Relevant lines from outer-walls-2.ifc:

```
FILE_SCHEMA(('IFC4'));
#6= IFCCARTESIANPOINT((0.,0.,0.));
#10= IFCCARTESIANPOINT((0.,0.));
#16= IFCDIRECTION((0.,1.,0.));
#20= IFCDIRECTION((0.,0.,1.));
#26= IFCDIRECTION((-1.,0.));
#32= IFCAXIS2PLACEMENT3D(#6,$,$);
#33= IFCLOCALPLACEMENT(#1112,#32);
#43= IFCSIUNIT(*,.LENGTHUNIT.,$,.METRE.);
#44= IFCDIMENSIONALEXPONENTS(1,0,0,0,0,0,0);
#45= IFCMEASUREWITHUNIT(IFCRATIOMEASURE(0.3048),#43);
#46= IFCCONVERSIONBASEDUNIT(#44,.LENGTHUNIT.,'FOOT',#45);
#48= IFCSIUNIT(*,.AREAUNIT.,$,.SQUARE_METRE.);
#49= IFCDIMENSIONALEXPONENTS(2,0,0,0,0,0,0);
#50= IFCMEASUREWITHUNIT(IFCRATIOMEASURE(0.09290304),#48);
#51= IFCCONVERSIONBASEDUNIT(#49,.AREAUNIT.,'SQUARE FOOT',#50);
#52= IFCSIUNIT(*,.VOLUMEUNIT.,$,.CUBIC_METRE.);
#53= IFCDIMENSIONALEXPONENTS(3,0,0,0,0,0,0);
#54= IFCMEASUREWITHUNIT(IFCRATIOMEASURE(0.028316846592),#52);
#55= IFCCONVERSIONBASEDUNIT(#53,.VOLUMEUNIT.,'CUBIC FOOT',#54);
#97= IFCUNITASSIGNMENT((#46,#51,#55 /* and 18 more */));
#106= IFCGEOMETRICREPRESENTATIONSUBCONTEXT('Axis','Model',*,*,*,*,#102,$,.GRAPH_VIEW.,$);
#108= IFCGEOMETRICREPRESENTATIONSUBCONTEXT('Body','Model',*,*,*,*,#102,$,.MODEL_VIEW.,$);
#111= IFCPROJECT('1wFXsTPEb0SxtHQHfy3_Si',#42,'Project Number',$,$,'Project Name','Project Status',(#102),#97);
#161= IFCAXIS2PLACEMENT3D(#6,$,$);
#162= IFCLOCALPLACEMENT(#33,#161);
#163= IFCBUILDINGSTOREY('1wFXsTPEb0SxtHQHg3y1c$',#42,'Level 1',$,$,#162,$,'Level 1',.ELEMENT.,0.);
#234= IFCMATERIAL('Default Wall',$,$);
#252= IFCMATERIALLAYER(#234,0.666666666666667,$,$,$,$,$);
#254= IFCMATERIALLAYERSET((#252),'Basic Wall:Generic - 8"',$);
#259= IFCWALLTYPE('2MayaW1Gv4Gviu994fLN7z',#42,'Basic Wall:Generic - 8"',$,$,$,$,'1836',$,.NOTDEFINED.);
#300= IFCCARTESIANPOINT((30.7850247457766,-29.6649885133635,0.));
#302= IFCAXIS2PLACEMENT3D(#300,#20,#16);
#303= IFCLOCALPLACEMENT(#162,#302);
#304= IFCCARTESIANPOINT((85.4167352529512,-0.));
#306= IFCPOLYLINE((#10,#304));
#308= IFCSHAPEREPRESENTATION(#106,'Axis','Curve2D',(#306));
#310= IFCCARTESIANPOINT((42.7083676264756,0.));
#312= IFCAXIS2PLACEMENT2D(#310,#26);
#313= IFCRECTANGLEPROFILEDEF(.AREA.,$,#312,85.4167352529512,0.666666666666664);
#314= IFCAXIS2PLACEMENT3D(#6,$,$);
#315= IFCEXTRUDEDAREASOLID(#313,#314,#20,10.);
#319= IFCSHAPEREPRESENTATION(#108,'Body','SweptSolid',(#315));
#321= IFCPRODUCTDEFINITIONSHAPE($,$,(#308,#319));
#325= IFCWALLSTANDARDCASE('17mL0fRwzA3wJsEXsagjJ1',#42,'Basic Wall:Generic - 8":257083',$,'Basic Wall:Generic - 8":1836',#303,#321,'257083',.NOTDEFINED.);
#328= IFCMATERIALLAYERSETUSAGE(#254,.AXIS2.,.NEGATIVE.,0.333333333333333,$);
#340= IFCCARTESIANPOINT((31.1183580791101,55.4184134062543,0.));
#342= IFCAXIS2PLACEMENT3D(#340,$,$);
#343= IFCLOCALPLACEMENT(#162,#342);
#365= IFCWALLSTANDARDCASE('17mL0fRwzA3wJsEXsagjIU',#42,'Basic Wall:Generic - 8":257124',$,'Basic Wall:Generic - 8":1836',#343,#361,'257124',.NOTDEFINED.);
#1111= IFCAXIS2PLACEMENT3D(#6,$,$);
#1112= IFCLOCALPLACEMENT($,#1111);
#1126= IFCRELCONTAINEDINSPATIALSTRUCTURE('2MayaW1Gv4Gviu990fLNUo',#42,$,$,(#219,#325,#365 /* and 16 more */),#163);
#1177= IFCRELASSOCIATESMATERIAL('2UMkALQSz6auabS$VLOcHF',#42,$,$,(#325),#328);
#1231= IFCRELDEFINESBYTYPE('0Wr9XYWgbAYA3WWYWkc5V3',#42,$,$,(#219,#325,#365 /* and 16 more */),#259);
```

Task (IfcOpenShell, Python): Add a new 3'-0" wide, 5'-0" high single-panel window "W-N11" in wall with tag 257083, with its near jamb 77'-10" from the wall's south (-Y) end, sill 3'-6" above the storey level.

```python
import numpy as np
import ifcopenshell
import ifcopenshell.api.feature
import ifcopenshell.api.geometry
import ifcopenshell.api.root
import ifcopenshell.api.spatial
import ifcopenshell.geom
import ifcopenshell.util.element
import ifcopenshell.util.placement
import ifcopenshell.util.representation
import ifcopenshell.util.shape
import ifcopenshell.util.unit

model = ifcopenshell.open("outer-walls-2.ifc")
unit_scale = ifcopenshell.util.unit.calculate_unit_scale(model)
settings = ifcopenshell.geom.settings()


def volume(element):
    """Net volume in cubic metres, openings subtracted."""
    shape = ifcopenshell.geom.create_shape(settings, element)
    return ifcopenshell.util.shape.get_volume(shape.geometry)


wall = model.by_guid("17mL0fRwzA3wJsEXsagjJ1")
storey = ifcopenshell.util.element.get_container(wall, ifc_class="IfcBuildingStorey")
context = ifcopenshell.util.representation.get_context(model, "Model", "Body", "MODEL_VIEW")
before = volume(wall)

width, height, from_end, sill = 0.9144, 1.524, 23.7236, 1.0668  # metres

# The wall runs along its own X axis, and the end named is its -X end.
wall_shape = ifcopenshell.geom.create_shape(settings, wall)
x, y, z = ifcopenshell.util.shape.get_vertices(wall_shape.geometry).T
start = x.min() + from_end
face, thickness = float(y.min()), float(y.max() - y.min())
wall_matrix = ifcopenshell.util.placement.get_local_placement(wall.ObjectPlacement)
level = ifcopenshell.util.placement.get_local_placement(storey.ObjectPlacement)[2, 3]


def in_wall(x, y):
    """Placement at x, y metres in the wall's axes, at sill height."""
    matrix = wall_matrix.copy()
    matrix[:, 3] = wall_matrix @ np.array([x / unit_scale, y / unit_scale, 0.0, 1.0])
    matrix[2, 3] = level + sill / unit_scale
    return matrix


# Opening: a box that overshoots both wall faces by 50 mm.
opening = ifcopenshell.api.root.create_entity(model, ifc_class="IfcOpeningElement", predefined_type="OPENING")
box = ifcopenshell.api.geometry.add_wall_representation(
    model, context=context, length=width, height=height, thickness=thickness + 0.1
)
ifcopenshell.api.geometry.assign_representation(model, product=opening, representation=box)
ifcopenshell.api.geometry.edit_object_placement(model, product=opening, matrix=in_wall(start, face - 0.05), is_si=False)
ifcopenshell.api.feature.add_feature(model, feature=opening, element=wall)

window = ifcopenshell.api.root.create_entity(model, ifc_class="IfcWindow", name="W-N11", predefined_type="WINDOW")
window.OverallWidth, window.OverallHeight = width / unit_scale, height / unit_scale
window.PartitioningType = "SINGLE_PANEL"
body = ifcopenshell.api.geometry.add_window_representation(
    model,
    context=context,
    overall_width=window.OverallWidth,
    overall_height=window.OverallHeight,
    partition_type="SINGLE_PANEL",
)
ifcopenshell.api.geometry.assign_representation(model, product=window, representation=body)
ifcopenshell.api.spatial.assign_container(model, products=[window], relating_structure=storey)
ifcopenshell.api.feature.add_filling(model, opening=opening, element=window)

# Centre the window in the wall's thickness.
ifcopenshell.api.geometry.edit_object_placement(model, product=window, matrix=in_wall(start, face), is_si=False)
window_shape = ifcopenshell.geom.create_shape(settings, window)
depth = ifcopenshell.util.shape.get_vertices(window_shape.geometry)[:, 1]
offset = face + thickness / 2 - (depth.min() + depth.max()) / 2
ifcopenshell.api.geometry.edit_object_placement(model, product=window, matrix=in_wall(start, offset), is_si=False)

after = volume(wall)

print(f"wall volume {before:.3f} -> {after:.3f} m3")

model.write("outer-walls-2_edited.ifc")
```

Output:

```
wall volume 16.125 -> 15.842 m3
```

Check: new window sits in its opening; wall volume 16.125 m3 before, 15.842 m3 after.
